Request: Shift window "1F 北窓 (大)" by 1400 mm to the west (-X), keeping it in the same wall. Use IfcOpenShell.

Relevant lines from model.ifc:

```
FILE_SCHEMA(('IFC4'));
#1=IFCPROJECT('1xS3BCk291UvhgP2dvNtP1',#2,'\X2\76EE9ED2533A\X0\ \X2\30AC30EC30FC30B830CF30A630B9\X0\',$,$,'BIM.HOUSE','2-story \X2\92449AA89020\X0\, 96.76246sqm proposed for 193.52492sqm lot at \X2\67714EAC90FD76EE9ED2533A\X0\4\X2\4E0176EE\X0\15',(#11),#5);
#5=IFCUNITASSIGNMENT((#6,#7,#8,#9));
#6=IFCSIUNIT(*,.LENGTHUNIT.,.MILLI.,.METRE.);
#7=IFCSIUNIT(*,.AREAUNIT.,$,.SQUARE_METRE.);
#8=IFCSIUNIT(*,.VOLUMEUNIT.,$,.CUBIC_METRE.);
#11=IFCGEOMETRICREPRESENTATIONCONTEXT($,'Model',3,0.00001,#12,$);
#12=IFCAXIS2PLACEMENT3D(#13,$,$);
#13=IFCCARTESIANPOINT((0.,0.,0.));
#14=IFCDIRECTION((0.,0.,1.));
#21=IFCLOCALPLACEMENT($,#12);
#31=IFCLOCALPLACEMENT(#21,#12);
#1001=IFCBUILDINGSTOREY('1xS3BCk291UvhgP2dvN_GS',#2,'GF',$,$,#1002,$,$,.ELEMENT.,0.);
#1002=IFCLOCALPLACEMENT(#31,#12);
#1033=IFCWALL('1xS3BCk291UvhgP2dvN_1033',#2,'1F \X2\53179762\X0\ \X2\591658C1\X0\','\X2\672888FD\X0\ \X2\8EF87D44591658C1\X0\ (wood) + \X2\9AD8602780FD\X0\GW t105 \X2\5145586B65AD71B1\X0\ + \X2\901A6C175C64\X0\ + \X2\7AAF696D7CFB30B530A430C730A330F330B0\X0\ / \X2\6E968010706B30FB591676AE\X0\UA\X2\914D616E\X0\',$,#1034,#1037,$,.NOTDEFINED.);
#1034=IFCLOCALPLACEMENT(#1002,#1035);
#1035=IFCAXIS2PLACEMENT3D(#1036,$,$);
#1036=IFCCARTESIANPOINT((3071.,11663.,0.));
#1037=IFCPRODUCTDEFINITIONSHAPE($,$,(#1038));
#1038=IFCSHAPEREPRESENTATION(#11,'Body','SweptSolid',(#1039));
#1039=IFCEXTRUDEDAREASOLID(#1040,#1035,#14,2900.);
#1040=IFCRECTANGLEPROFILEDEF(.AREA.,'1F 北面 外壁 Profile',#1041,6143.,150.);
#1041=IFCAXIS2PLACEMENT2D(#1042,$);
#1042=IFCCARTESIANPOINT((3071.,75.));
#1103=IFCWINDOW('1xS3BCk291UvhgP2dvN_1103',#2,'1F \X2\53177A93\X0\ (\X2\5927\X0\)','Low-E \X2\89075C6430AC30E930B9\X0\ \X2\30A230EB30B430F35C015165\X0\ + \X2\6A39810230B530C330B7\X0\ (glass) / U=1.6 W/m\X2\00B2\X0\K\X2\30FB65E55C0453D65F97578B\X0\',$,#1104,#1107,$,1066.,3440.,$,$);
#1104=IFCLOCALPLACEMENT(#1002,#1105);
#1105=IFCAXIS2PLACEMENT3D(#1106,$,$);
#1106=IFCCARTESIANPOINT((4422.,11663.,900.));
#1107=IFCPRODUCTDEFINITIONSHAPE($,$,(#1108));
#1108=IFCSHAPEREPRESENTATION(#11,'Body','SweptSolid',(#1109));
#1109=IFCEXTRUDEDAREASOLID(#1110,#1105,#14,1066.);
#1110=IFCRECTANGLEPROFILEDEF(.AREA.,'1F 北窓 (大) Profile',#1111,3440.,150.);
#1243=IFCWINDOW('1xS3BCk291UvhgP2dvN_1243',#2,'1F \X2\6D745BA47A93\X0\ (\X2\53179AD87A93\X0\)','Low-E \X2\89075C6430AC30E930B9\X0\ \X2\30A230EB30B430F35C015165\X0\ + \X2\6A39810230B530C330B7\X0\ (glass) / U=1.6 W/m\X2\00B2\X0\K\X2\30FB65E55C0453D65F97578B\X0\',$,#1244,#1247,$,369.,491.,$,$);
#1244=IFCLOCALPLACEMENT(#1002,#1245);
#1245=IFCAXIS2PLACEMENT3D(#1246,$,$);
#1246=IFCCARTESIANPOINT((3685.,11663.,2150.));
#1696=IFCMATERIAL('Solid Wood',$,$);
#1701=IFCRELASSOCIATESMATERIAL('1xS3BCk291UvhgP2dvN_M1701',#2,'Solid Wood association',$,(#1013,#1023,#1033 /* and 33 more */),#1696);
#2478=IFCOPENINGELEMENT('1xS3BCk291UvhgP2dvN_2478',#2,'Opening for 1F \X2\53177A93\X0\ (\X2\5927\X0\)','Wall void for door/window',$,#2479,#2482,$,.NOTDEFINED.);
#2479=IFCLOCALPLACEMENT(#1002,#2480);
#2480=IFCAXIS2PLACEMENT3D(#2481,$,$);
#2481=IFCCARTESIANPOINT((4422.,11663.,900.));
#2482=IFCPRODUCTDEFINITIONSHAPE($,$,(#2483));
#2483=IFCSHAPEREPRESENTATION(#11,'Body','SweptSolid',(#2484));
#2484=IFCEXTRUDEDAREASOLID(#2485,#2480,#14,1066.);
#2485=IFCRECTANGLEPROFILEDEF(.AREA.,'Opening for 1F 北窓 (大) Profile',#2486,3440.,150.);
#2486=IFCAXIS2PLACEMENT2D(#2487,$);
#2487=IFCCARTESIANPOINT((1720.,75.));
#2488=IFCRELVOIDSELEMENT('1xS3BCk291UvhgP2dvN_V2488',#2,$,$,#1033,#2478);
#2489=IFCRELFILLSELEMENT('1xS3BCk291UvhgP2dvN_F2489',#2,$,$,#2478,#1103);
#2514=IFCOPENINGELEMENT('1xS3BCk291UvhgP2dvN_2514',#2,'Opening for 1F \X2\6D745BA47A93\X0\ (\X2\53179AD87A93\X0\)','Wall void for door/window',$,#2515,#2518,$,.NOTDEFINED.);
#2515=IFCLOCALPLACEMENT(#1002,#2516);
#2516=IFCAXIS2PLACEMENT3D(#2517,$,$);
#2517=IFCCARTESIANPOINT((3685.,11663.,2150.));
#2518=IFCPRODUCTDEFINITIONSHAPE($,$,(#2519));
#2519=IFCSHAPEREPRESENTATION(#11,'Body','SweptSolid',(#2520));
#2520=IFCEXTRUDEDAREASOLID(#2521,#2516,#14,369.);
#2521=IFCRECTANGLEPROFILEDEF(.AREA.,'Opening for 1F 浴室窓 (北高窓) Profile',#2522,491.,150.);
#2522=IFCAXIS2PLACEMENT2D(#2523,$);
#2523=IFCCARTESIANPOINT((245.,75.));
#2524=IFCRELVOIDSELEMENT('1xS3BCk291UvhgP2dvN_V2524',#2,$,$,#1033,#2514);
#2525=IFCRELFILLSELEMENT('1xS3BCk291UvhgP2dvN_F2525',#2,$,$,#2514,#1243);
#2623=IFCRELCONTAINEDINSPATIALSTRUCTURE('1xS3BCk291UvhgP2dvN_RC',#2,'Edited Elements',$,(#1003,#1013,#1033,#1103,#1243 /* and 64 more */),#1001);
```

```python
import ifcopenshell
import ifcopenshell.api.geometry
import ifcopenshell.util.placement
import ifcopenshell.util.unit

model = ifcopenshell.open("model.ifc")
unit_scale = ifcopenshell.util.unit.calculate_unit_scale(model)

window = model.by_guid("1xS3BCk291UvhgP2dvN_1103")
opening = window.FillsVoids[0].RelatingOpeningElement
wall = opening.VoidsElements[0].RelatingBuildingElement

wall_matrix = ifcopenshell.util.placement.get_local_placement(wall.ObjectPlacement)
shift = wall_matrix[:3, 0] * -1.4 / unit_scale
before = ifcopenshell.util.placement.get_local_placement(window.ObjectPlacement)[:3, 3].copy()

# The window is not placed relative to its opening, so move both.
for product in (opening, window):
    matrix = ifcopenshell.util.placement.get_local_placement(product.ObjectPlacement)
    matrix[:3, 3] += shift
    ifcopenshell.api.geometry.edit_object_placement(model, product=product, matrix=matrix, is_si=False)

after = ifcopenshell.util.placement.get_local_placement(window.ObjectPlacement)[:3, 3]
print("window moved by", (after - before).round(3) + 0.0)

model.write("model_updated.ifc")
```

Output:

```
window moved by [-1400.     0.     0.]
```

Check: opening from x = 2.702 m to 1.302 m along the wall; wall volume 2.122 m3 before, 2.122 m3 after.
